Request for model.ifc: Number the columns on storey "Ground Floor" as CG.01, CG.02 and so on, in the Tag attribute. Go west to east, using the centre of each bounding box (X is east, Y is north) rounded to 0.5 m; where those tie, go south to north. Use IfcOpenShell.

First a look at what the model holds.

```python
import ifcopenshell
import ifcopenshell.util.element
import ifcopenshell.util.placement

model = ifcopenshell.open("model.ifc")
print(model.schema)
storey = next(s for s in model.by_type("IfcBuildingStorey") if s.Name == "Ground Floor")
columns = [e for e in ifcopenshell.util.element.get_decomposition(storey) if e.is_a("IfcColumn")]
for e in sorted(columns, key=lambda e: e.id()):
    origin = ifcopenshell.util.placement.get_local_placement(e.ObjectPlacement)[:3, 3]
    print(e.id(), e.Tag, e.Name, origin.round(2) + 0.0, sep=" | ")
```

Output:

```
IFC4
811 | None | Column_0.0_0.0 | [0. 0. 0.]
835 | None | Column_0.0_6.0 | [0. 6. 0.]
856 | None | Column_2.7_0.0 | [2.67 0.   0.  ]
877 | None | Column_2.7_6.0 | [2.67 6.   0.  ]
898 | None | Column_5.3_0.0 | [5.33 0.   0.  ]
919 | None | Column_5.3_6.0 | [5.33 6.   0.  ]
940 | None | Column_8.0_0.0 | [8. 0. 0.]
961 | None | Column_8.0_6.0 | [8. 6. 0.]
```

```python
import ifcopenshell
import ifcopenshell.geom
import ifcopenshell.util.element
import ifcopenshell.util.shape

model = ifcopenshell.open("model.ifc")
settings = ifcopenshell.geom.settings()
settings.set("use-world-coords", True)


def centre(element):
    shape = ifcopenshell.geom.create_shape(settings, element)
    return ifcopenshell.util.shape.get_bbox_centroid(shape.geometry)


storey = next(s for s in model.by_type("IfcBuildingStorey") if s.Name == "Ground Floor")
columns = [e for e in ifcopenshell.util.element.get_decomposition(storey) if e.is_a("IfcColumn")]

# Insertion points can sit at a corner or the storey origin, so sort by the geometry (in metres).
centres = {e: centre(e) for e in columns}
columns.sort(key=lambda e: (round(centres[e][0] / 0.5), centres[e][1]))

for i, e in enumerate(columns, start=1):
    number = f"CG.{i:02d}"
    e.Tag = number
    print(e.id(), number)

model.write("model-out.ifc")
```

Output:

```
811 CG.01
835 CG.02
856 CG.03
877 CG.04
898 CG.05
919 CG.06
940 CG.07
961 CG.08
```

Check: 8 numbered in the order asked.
